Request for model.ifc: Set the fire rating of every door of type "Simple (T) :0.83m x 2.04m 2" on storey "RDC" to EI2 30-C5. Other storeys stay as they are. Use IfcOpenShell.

First a look at what the model holds.

```python
import ifcopenshell
import ifcopenshell.util.element

model = ifcopenshell.open("model.ifc")
print(model.schema)
storey = next(s for s in model.by_type("IfcBuildingStorey") if s.Name == "RDC")
doors = [e for e in ifcopenshell.util.element.get_decomposition(storey) if e.is_a("IfcDoor")]
seen = {}
for e in doors:
    element_type = ifcopenshell.util.element.get_type(e)
    key = (element_type.Name if element_type != e and element_type else None, ifcopenshell.util.element.get_pset(e, "Pset_DoorCommon", "FireRating"))
    seen[key] = seen.get(key, 0) + 1
for (name, value), count in sorted(seen.items(), key=str):
    print(count, "x", name, "|", value)
```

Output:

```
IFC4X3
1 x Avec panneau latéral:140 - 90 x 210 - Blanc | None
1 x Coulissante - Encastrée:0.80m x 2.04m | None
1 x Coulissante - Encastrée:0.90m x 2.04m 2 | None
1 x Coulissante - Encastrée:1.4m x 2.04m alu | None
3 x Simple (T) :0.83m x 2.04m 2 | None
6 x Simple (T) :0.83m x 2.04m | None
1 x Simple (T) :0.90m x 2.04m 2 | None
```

```python
import ifcopenshell
import ifcopenshell.api.pset
import ifcopenshell.util.element

model = ifcopenshell.open("model.ifc")

storey = next(s for s in model.by_type("IfcBuildingStorey") if s.Name == "RDC")
doors = [e for e in ifcopenshell.util.element.get_decomposition(storey) if e.is_a("IfcDoor")]

count = 0
for e in doors:
    element_type = ifcopenshell.util.element.get_type(e)
    if element_type in (None, e) or element_type.Name != "Simple (T) :0.83m x 2.04m 2":
        continue
    # add_pset returns the element's existing set when there is one.
    pset = ifcopenshell.api.pset.add_pset(model, product=e, name="Pset_DoorCommon")
    ifcopenshell.api.pset.edit_pset(model, pset=pset, properties={"FireRating": "EI2 30-C5"})
    count += 1

print(count, "doors updated")

model.write("model_v2.ifc")
```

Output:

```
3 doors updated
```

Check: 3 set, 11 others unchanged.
